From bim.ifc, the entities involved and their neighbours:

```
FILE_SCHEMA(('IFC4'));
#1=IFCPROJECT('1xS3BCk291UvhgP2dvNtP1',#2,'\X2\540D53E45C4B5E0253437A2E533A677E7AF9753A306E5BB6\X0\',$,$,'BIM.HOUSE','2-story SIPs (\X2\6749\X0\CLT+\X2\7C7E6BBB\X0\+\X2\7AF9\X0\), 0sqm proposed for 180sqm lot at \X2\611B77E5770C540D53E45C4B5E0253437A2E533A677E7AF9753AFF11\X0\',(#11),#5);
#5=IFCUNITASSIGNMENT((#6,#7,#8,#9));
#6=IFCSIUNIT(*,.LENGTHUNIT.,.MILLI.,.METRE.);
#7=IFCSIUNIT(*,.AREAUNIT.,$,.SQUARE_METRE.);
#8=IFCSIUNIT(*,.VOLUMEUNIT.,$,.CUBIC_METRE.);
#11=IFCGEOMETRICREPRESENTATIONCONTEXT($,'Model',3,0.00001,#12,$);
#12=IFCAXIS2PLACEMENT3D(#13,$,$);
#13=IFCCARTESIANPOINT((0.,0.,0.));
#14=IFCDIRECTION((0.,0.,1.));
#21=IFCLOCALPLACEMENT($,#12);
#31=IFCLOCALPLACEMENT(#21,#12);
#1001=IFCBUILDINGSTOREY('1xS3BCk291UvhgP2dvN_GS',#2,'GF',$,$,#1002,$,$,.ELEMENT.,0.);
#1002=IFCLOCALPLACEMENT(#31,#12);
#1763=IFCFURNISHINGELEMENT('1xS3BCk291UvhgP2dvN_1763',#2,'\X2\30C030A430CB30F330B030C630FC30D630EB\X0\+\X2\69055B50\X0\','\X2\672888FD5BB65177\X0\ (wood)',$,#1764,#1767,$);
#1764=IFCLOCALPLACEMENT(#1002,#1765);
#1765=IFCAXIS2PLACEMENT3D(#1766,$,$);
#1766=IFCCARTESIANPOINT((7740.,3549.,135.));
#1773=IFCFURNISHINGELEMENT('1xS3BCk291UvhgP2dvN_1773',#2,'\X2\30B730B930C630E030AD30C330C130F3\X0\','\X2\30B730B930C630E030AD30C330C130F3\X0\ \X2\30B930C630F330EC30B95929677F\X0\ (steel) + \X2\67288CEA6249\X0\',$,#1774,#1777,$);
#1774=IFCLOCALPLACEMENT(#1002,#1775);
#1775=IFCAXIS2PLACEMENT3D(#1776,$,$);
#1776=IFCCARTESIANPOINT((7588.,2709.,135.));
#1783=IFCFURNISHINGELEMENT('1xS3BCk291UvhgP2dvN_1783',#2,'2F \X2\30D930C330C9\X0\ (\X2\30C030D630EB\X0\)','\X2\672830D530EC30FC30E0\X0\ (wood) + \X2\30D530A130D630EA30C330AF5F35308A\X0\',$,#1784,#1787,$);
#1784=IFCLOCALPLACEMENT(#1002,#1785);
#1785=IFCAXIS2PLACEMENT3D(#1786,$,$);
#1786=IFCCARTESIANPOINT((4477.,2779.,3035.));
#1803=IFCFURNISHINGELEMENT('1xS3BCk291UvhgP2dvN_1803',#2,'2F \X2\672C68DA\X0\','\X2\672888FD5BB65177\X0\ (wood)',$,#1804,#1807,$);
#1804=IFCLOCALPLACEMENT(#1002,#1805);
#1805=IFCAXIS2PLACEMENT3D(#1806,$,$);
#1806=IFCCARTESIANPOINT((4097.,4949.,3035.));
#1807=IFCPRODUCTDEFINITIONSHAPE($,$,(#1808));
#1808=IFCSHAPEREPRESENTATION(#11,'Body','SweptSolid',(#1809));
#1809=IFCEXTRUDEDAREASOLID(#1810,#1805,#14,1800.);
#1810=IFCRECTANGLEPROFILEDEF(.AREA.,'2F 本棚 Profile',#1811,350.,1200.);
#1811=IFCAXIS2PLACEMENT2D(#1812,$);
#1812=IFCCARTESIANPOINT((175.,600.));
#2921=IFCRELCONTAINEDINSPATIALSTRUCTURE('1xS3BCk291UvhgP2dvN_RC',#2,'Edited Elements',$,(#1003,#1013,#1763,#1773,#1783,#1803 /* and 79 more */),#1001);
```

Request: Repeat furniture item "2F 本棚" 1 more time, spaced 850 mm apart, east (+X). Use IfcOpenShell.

```python
import numpy as np
import ifcopenshell
import ifcopenshell.api.geometry
import ifcopenshell.api.root
import ifcopenshell.util.element
import ifcopenshell.util.placement
import ifcopenshell.util.unit

model = ifcopenshell.open("bim.ifc")
unit_scale = ifcopenshell.util.unit.calculate_unit_scale(model)


def reuse_history(source, copy):
    """copy_class also copies each property set's owner history, people and application; keep the originals."""
    for rel in copy.IsDefinedBy:
        if rel.is_a("IfcRelDefinesByProperties") and (history := rel.RelatingPropertyDefinition.OwnerHistory):
            rel.RelatingPropertyDefinition.OwnerHistory = source.OwnerHistory
            ifcopenshell.util.element.remove_deep2(model, history)


source = model.by_id(1803)
base = ifcopenshell.util.placement.get_local_placement(source.ObjectPlacement)
step = np.array([1.0, 0.0, 0.0]) * 0.85 / unit_scale

for i in range(1, 2):
    copy = ifcopenshell.api.root.copy_class(model, product=source)
    copy.Representation = ifcopenshell.util.element.copy_deep(
        model, source.Representation, exclude=["IfcGeometricRepresentationContext", "IfcRepresentationMap"]
    )
    reuse_history(source, copy)
    matrix = base.copy()
    matrix[:3, 3] += i * step
    print("added at", matrix[:3, 3].round(3) + 0.0)
    ifcopenshell.api.geometry.edit_object_placement(model, product=copy, matrix=matrix, is_si=False)

model.write("bim_updated.ifc")
```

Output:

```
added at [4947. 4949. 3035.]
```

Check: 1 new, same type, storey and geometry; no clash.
